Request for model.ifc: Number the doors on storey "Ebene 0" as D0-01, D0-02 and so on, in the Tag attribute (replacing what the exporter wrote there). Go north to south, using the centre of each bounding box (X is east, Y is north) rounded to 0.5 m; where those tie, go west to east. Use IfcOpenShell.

First a look at what the model holds.

```python
import ifcopenshell
import ifcopenshell.util.element
import ifcopenshell.util.placement

model = ifcopenshell.open("model.ifc")
print(model.schema)
storey = next(s for s in model.by_type("IfcBuildingStorey") if s.Name == "Ebene 0")
doors = [e for e in ifcopenshell.util.element.get_decomposition(storey) if e.is_a("IfcDoor")]
for e in sorted(doors, key=lambda e: e.id()):
    origin = ifcopenshell.util.placement.get_local_placement(e.ObjectPlacement)[:3, 3]
    print(e.id(), e.Tag, e.Name, origin.round(2) + 0.0, sep=" | ")
```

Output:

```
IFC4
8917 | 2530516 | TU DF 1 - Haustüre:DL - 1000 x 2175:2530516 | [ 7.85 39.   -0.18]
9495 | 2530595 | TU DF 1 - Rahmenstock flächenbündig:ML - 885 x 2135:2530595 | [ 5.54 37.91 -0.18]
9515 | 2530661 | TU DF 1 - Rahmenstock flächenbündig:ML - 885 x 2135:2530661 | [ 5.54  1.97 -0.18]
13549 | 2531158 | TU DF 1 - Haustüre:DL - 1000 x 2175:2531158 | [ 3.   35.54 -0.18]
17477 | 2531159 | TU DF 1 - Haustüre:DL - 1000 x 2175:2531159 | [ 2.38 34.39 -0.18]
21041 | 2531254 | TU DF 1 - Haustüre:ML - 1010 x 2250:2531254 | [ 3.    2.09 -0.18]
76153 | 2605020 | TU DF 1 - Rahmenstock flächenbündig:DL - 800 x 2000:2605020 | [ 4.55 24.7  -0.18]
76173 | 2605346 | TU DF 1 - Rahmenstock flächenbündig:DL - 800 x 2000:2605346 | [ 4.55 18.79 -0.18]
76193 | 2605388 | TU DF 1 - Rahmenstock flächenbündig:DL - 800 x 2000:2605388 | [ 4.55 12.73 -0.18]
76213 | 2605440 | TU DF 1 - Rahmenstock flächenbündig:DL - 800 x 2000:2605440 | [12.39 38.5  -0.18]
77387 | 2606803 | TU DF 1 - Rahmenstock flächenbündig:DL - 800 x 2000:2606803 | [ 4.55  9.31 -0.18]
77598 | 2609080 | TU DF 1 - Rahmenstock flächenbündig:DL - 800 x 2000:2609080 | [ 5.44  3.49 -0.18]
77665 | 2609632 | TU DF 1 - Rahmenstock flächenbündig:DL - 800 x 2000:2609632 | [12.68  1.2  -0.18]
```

```python
import ifcopenshell
import ifcopenshell.geom
import ifcopenshell.util.element
import ifcopenshell.util.shape

model = ifcopenshell.open("model.ifc")
settings = ifcopenshell.geom.settings()
settings.set("use-world-coords", True)


def centre(element):
    shape = ifcopenshell.geom.create_shape(settings, element)
    return ifcopenshell.util.shape.get_bbox_centroid(shape.geometry)


storey = next(s for s in model.by_type("IfcBuildingStorey") if s.Name == "Ebene 0")
doors = [e for e in ifcopenshell.util.element.get_decomposition(storey) if e.is_a("IfcDoor")]

# Insertion points can sit at a corner or the storey origin, so sort by the geometry (in metres).
centres = {e: centre(e) for e in doors}
doors.sort(key=lambda e: (-round(centres[e][1] / 0.5), centres[e][0]))

for i, e in enumerate(doors, start=1):
    number = f"D0-{i:02d}"
    e.Tag = number
    print(e.id(), number)

model.write("model_edited.ifc")
```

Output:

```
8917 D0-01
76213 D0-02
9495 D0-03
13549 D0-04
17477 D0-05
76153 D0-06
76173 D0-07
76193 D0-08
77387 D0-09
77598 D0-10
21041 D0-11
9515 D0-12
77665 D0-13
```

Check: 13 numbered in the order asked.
